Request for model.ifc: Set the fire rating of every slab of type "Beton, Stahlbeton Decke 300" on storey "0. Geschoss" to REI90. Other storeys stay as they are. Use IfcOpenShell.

First a look at what the model holds.

```python
import ifcopenshell
import ifcopenshell.util.element

model = ifcopenshell.open("model.ifc")
print(model.schema)
storey = next(s for s in model.by_type("IfcBuildingStorey") if s.Name == "0. Geschoss")
slabs = [e for e in ifcopenshell.util.element.get_decomposition(storey) if e.is_a("IfcSlab")]
seen = {}
for e in slabs:
    element_type = ifcopenshell.util.element.get_type(e)
    key = (element_type.Name if element_type != e and element_type else None, ifcopenshell.util.element.get_pset(e, "Pset_SlabCommon", "FireRating"))
    seen[key] = seen.get(key, 0) + 1
for (name, value), count in sorted(seen.items(), key=str):
    print(count, "x", name, "|", value)
```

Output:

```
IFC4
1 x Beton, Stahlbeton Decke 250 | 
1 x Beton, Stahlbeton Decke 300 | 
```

```python
import ifcopenshell
import ifcopenshell.api.pset
import ifcopenshell.util.element

model = ifcopenshell.open("model.ifc")

storey = next(s for s in model.by_type("IfcBuildingStorey") if s.Name == "0. Geschoss")
slabs = [e for e in ifcopenshell.util.element.get_decomposition(storey) if e.is_a("IfcSlab")]

count = 0
for e in slabs:
    element_type = ifcopenshell.util.element.get_type(e)
    if element_type in (None, e) or element_type.Name != "Beton, Stahlbeton Decke 300":
        continue
    # add_pset returns the element's existing set when there is one.
    pset = ifcopenshell.api.pset.add_pset(model, product=e, name="Pset_SlabCommon")
    ifcopenshell.api.pset.edit_pset(model, pset=pset, properties={"FireRating": "REI90"})
    count += 1

print(count, "slabs updated")

model.write("model-out.ifc")
```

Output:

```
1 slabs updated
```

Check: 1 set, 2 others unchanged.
